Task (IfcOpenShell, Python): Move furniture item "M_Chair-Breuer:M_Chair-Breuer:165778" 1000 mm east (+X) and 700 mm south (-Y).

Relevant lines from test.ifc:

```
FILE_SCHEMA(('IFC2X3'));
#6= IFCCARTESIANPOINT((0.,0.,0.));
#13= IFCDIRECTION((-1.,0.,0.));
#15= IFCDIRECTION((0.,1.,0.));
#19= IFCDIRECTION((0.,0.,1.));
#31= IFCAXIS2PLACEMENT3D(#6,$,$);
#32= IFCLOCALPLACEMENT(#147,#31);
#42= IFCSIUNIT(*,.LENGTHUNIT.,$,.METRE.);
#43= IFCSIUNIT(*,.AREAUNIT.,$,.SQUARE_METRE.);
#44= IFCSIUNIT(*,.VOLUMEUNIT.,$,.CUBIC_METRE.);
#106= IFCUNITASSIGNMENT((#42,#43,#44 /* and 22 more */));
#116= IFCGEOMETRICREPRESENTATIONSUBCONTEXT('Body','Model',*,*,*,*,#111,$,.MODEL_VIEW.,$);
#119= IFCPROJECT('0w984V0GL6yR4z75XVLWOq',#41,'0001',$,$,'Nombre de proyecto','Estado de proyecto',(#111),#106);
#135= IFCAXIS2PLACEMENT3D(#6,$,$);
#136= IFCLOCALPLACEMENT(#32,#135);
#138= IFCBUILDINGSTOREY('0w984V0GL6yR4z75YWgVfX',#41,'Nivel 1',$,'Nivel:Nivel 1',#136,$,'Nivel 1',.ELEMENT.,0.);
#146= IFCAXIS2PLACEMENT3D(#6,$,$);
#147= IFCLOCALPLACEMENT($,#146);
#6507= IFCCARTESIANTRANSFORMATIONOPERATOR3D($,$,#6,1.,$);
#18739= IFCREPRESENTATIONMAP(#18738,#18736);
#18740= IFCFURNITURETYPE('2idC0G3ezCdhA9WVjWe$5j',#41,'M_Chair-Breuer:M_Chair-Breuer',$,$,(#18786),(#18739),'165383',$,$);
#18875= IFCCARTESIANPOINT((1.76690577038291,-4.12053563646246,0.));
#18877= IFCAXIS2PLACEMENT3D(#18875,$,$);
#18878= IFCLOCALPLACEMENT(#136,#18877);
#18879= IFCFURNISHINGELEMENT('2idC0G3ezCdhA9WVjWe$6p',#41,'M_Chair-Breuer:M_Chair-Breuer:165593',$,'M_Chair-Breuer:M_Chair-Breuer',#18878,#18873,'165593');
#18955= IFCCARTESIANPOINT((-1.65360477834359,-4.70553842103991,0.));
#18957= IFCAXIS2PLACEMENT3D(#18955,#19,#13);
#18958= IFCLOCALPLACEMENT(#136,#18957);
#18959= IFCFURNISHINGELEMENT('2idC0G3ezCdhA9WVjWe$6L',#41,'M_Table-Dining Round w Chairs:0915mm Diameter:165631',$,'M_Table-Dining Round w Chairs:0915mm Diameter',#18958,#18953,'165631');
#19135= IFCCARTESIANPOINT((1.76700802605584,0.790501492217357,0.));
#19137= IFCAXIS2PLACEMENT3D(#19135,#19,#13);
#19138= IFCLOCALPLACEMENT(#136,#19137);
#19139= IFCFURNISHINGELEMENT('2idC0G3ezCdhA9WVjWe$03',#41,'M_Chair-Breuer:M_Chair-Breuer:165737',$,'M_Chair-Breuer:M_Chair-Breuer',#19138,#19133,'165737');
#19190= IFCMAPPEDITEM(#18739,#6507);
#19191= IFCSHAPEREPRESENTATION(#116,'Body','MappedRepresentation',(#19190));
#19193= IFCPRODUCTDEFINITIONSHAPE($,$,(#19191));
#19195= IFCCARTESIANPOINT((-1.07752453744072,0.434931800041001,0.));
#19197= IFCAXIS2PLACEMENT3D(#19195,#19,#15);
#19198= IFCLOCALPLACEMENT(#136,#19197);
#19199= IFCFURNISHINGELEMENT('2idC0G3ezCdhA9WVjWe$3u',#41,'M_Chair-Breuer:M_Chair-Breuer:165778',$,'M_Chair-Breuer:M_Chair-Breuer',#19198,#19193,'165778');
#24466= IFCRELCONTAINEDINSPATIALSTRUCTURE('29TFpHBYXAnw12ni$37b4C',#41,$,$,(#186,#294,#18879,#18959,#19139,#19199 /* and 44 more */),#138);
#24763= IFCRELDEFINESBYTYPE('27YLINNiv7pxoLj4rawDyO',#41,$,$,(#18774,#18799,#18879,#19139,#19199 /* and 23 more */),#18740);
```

```python
import ifcopenshell
import ifcopenshell.api.geometry
import ifcopenshell.util.placement
import ifcopenshell.util.unit

model = ifcopenshell.open("test.ifc")
unit_scale = ifcopenshell.util.unit.calculate_unit_scale(model)

item = model.by_guid("2idC0G3ezCdhA9WVjWe$3u")
matrix = ifcopenshell.util.placement.get_local_placement(item.ObjectPlacement)
matrix[0, 3] += 1 / unit_scale
matrix[1, 3] -= 0.7 / unit_scale
ifcopenshell.api.geometry.edit_object_placement(model, product=item, matrix=matrix, is_si=False)

print(ifcopenshell.util.placement.get_local_placement(item.ObjectPlacement).round(3) + 0.0)

model.write("test_rev.ifc")
```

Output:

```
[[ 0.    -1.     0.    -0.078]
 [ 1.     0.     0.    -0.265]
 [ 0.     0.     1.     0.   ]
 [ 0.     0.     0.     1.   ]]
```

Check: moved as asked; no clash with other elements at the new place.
